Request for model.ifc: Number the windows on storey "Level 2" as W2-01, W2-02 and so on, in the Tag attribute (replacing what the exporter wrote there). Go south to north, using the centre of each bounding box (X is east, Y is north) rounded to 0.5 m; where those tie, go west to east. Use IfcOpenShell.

First a look at what the model holds.

```python
import ifcopenshell
import ifcopenshell.util.element
import ifcopenshell.util.placement

model = ifcopenshell.open("model.ifc")
print(model.schema)
storey = next(s for s in model.by_type("IfcBuildingStorey") if s.Name == "Level 2")
windows = [e for e in ifcopenshell.util.element.get_decomposition(storey) if e.is_a("IfcWindow")]
for e in sorted(windows, key=lambda e: e.id()):
    origin = ifcopenshell.util.placement.get_local_placement(e.ObjectPlacement)[:3, 3]
    print(e.id(), e.Tag, e.Name, origin.round(2) + 0.0, sep=" | ")
```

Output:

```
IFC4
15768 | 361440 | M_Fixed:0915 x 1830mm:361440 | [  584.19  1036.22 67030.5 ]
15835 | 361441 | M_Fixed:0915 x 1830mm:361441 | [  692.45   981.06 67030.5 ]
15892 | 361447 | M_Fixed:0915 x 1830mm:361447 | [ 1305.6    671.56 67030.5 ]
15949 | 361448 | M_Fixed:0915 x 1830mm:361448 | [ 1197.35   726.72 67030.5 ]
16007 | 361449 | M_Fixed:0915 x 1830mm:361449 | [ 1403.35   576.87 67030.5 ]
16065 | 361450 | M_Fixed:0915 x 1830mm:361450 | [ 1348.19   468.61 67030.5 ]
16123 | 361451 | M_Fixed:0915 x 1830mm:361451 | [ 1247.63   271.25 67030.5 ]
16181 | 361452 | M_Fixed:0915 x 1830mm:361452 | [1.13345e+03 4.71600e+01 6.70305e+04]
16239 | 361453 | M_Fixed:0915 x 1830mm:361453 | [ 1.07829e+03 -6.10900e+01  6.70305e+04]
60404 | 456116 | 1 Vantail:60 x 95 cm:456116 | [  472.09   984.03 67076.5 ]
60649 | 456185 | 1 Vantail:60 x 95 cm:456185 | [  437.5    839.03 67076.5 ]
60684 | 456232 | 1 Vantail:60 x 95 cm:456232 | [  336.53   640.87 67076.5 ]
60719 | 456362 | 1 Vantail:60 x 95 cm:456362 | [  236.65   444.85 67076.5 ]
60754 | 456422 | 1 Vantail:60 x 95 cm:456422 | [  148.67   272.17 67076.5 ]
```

```python
import ifcopenshell
import ifcopenshell.geom
import ifcopenshell.util.element
import ifcopenshell.util.shape

model = ifcopenshell.open("model.ifc")
settings = ifcopenshell.geom.settings()
settings.set("use-world-coords", True)


def centre(element):
    shape = ifcopenshell.geom.create_shape(settings, element)
    return ifcopenshell.util.shape.get_bbox_centroid(shape.geometry)


storey = next(s for s in model.by_type("IfcBuildingStorey") if s.Name == "Level 2")
windows = [e for e in ifcopenshell.util.element.get_decomposition(storey) if e.is_a("IfcWindow")]

# Insertion points can sit at a corner or the storey origin, so sort by the geometry (in metres).
centres = {e: centre(e) for e in windows}
windows.sort(key=lambda e: (round(centres[e][1] / 0.5), centres[e][0]))

for i, e in enumerate(windows, start=1):
    number = f"W2-{i:02d}"
    e.Tag = number
    print(e.id(), number)

model.write("model_edited.ifc")
```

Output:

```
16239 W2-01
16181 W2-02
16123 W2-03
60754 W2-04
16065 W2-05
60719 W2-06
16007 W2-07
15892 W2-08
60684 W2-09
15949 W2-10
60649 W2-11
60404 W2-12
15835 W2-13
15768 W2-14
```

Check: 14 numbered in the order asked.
